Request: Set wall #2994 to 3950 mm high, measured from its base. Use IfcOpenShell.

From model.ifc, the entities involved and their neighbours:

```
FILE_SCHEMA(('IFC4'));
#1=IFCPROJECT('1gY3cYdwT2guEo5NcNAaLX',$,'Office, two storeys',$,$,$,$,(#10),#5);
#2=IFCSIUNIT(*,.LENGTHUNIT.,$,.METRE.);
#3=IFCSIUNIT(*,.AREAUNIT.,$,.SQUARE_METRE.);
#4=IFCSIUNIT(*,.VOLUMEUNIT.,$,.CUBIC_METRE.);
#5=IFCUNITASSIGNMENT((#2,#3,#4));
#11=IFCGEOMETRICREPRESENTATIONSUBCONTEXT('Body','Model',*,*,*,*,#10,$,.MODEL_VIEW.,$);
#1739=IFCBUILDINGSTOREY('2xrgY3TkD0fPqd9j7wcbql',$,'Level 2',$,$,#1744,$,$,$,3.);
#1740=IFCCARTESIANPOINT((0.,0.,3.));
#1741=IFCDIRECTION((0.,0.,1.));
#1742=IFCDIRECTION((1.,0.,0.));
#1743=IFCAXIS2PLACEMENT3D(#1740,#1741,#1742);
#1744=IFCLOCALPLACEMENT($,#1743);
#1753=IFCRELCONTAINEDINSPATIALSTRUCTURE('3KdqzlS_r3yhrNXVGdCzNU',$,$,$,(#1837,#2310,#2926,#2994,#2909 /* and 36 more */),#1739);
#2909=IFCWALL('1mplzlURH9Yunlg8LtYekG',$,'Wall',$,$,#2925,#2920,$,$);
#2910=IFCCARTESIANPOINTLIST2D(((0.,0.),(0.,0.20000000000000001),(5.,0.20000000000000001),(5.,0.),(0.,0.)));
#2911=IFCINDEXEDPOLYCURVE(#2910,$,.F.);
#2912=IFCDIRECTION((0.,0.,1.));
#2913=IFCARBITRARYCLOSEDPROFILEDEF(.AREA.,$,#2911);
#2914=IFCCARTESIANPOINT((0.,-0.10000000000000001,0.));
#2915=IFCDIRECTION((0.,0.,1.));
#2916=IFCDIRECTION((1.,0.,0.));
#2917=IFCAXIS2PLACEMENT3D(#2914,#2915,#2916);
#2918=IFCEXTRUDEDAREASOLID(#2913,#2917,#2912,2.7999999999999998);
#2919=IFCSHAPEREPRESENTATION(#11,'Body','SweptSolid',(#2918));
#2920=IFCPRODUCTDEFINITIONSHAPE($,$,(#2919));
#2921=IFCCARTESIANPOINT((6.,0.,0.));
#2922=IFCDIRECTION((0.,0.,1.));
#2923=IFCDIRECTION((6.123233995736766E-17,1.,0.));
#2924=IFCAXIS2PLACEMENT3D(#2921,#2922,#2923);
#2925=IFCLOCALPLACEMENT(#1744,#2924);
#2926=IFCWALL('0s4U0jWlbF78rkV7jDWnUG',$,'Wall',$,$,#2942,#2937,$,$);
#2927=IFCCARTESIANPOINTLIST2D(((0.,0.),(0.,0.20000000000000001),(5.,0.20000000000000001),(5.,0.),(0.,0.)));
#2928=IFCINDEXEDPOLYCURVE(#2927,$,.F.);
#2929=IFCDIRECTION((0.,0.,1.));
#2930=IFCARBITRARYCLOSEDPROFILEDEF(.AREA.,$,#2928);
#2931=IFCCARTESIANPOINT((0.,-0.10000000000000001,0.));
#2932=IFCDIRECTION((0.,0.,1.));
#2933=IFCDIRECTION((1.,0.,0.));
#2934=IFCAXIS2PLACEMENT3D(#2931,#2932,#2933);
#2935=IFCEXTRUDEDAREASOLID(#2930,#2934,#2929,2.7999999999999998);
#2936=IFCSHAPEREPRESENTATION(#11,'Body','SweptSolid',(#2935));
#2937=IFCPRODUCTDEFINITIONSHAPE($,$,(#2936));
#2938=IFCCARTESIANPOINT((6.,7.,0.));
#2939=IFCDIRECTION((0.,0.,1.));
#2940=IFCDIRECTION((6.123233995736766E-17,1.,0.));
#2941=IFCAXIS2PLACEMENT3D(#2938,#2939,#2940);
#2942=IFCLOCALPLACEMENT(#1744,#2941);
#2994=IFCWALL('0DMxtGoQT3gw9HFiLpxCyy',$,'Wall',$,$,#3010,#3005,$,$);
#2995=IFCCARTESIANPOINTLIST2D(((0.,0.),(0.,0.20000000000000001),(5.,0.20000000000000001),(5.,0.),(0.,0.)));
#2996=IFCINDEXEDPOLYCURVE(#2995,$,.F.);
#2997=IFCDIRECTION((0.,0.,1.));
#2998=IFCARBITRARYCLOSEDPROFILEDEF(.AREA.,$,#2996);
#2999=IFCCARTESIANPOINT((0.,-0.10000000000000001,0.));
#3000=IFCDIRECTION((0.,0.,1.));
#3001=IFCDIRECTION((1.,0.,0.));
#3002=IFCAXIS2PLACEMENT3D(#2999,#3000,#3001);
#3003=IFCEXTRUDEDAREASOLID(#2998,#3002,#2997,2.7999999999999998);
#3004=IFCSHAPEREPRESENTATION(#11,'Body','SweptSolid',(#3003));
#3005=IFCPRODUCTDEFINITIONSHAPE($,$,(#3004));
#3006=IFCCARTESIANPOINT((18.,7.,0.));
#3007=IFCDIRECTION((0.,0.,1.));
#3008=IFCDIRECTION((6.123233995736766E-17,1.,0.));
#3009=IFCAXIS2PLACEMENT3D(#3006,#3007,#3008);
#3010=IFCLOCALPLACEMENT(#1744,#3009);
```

```python
import ifcopenshell
import ifcopenshell.geom
import ifcopenshell.util.representation
import ifcopenshell.util.shape
import ifcopenshell.util.unit

model = ifcopenshell.open("model.ifc")
unit_scale = ifcopenshell.util.unit.calculate_unit_scale(model)
settings = ifcopenshell.geom.settings()


def volume(element):
    """Net volume in cubic metres, openings subtracted."""
    shape = ifcopenshell.geom.create_shape(settings, element)
    return ifcopenshell.util.shape.get_volume(shape.geometry)


wall = model.by_id(2994)
before = volume(wall)

body = ifcopenshell.util.representation.get_representation(wall, "Model", "Body")
solid = body.Items[0]
old_height = solid.Depth
solid.Depth = 3.95 / unit_scale
after = volume(wall)

print(f"height {old_height:g} -> {solid.Depth:g}, volume {before:.3f} -> {after:.3f} m3")

model.write("model-out.ifc")
```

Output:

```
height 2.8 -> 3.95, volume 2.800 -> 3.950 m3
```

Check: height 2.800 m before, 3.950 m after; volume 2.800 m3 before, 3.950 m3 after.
